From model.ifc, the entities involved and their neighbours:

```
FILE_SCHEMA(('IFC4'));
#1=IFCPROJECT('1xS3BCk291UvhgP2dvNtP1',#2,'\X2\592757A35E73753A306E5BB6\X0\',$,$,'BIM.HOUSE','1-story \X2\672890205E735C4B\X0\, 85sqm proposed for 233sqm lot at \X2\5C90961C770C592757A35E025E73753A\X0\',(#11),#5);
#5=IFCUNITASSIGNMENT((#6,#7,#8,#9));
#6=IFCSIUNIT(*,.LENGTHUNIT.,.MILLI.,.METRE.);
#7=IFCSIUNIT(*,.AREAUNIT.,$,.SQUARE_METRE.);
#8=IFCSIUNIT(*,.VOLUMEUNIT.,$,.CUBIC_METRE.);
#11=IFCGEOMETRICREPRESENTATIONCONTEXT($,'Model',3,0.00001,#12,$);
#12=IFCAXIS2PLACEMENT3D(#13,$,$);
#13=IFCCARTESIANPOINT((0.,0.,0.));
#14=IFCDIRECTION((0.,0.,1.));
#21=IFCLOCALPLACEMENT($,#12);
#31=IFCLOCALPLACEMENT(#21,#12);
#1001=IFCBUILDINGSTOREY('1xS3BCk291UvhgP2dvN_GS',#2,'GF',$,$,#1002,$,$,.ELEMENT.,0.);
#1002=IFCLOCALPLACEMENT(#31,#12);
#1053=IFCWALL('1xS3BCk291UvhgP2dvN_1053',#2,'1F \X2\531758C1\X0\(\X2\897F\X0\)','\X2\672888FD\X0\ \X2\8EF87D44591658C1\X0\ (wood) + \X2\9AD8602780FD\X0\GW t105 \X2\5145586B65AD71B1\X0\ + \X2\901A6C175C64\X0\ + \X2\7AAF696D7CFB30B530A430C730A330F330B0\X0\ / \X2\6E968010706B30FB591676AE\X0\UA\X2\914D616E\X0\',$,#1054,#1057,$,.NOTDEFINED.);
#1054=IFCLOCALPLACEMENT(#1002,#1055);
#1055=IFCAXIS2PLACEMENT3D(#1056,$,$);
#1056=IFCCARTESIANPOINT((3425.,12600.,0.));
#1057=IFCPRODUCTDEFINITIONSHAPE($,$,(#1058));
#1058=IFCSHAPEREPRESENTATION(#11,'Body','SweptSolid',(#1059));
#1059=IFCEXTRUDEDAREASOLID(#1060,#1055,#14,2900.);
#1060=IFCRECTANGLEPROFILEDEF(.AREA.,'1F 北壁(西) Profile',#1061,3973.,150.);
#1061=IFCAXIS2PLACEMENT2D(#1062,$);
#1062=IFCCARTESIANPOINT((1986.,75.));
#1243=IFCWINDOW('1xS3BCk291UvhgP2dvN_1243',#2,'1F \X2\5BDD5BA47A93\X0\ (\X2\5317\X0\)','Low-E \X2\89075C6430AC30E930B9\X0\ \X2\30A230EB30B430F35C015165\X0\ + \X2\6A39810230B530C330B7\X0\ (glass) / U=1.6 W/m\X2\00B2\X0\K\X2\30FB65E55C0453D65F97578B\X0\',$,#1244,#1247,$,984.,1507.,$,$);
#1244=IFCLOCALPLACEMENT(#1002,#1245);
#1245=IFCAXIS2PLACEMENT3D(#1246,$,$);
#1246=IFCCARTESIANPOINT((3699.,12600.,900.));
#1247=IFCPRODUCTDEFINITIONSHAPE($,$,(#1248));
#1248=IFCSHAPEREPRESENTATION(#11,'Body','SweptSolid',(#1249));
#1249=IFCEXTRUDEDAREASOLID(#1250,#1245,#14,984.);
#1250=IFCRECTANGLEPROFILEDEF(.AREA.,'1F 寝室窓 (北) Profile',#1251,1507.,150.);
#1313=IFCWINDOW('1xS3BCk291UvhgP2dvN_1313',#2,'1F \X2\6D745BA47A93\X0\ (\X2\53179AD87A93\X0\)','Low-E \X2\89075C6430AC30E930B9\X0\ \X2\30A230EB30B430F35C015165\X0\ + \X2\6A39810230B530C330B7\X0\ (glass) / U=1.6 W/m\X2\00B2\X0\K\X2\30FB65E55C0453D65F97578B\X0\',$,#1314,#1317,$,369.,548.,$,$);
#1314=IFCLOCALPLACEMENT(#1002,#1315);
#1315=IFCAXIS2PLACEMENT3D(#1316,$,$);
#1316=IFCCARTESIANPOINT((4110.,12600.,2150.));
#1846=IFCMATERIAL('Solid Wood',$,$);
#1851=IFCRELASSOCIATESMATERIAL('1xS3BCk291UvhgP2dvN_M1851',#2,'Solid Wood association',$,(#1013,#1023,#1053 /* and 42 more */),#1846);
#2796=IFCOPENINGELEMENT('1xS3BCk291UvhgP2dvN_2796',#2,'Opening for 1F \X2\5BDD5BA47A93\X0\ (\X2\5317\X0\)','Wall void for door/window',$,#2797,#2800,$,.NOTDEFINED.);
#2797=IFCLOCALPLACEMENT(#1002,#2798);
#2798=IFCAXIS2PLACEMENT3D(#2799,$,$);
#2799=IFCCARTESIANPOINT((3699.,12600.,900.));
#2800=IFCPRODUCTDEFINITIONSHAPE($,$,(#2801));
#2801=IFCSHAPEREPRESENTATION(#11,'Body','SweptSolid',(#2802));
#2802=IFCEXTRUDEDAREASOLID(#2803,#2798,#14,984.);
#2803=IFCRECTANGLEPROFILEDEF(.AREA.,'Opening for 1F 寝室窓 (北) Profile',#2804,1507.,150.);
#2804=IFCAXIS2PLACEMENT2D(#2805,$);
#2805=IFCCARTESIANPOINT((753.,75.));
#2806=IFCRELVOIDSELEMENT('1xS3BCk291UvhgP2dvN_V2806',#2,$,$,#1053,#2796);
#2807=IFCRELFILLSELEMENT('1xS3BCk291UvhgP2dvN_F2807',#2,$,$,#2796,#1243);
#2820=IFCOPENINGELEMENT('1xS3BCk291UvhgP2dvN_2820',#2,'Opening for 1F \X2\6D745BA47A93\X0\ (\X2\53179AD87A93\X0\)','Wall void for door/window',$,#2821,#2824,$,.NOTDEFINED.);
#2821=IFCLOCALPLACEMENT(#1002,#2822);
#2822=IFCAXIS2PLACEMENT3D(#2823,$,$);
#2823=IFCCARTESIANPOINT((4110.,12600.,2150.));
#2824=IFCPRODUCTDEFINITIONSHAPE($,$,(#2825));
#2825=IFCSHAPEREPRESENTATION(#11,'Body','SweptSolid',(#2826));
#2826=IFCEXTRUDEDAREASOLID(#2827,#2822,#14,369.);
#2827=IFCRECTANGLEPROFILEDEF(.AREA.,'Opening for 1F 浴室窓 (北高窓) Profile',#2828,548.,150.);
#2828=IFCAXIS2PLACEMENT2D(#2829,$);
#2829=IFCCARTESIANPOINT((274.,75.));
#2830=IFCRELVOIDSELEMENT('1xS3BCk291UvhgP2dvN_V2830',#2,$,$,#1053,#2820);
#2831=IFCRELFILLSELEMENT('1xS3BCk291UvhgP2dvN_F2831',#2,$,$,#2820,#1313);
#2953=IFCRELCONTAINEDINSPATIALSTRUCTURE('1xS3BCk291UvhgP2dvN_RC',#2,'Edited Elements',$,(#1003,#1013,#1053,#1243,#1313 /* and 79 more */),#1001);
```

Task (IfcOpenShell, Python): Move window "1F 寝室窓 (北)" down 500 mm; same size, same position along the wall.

```python
import numpy as np
import ifcopenshell
import ifcopenshell.api.geometry
import ifcopenshell.util.placement
import ifcopenshell.util.unit

model = ifcopenshell.open("model.ifc")
unit_scale = ifcopenshell.util.unit.calculate_unit_scale(model)

window = model.by_guid("1xS3BCk291UvhgP2dvN_1243")
opening = window.FillsVoids[0].RelatingOpeningElement
dz = -0.5 / unit_scale

shift = np.array([0.0, 0.0, dz])
# The window is not placed relative to its opening, so move both.
for product in (opening, window):
    matrix = ifcopenshell.util.placement.get_local_placement(product.ObjectPlacement)
    matrix[:3, 3] += shift
    ifcopenshell.api.geometry.edit_object_placement(model, product=product, matrix=matrix, is_si=False)

print(f"moved by {dz * unit_scale:+.3f} m")

model.write("model_edited.ifc")
```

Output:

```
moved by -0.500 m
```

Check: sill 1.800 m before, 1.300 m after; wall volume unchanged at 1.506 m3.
